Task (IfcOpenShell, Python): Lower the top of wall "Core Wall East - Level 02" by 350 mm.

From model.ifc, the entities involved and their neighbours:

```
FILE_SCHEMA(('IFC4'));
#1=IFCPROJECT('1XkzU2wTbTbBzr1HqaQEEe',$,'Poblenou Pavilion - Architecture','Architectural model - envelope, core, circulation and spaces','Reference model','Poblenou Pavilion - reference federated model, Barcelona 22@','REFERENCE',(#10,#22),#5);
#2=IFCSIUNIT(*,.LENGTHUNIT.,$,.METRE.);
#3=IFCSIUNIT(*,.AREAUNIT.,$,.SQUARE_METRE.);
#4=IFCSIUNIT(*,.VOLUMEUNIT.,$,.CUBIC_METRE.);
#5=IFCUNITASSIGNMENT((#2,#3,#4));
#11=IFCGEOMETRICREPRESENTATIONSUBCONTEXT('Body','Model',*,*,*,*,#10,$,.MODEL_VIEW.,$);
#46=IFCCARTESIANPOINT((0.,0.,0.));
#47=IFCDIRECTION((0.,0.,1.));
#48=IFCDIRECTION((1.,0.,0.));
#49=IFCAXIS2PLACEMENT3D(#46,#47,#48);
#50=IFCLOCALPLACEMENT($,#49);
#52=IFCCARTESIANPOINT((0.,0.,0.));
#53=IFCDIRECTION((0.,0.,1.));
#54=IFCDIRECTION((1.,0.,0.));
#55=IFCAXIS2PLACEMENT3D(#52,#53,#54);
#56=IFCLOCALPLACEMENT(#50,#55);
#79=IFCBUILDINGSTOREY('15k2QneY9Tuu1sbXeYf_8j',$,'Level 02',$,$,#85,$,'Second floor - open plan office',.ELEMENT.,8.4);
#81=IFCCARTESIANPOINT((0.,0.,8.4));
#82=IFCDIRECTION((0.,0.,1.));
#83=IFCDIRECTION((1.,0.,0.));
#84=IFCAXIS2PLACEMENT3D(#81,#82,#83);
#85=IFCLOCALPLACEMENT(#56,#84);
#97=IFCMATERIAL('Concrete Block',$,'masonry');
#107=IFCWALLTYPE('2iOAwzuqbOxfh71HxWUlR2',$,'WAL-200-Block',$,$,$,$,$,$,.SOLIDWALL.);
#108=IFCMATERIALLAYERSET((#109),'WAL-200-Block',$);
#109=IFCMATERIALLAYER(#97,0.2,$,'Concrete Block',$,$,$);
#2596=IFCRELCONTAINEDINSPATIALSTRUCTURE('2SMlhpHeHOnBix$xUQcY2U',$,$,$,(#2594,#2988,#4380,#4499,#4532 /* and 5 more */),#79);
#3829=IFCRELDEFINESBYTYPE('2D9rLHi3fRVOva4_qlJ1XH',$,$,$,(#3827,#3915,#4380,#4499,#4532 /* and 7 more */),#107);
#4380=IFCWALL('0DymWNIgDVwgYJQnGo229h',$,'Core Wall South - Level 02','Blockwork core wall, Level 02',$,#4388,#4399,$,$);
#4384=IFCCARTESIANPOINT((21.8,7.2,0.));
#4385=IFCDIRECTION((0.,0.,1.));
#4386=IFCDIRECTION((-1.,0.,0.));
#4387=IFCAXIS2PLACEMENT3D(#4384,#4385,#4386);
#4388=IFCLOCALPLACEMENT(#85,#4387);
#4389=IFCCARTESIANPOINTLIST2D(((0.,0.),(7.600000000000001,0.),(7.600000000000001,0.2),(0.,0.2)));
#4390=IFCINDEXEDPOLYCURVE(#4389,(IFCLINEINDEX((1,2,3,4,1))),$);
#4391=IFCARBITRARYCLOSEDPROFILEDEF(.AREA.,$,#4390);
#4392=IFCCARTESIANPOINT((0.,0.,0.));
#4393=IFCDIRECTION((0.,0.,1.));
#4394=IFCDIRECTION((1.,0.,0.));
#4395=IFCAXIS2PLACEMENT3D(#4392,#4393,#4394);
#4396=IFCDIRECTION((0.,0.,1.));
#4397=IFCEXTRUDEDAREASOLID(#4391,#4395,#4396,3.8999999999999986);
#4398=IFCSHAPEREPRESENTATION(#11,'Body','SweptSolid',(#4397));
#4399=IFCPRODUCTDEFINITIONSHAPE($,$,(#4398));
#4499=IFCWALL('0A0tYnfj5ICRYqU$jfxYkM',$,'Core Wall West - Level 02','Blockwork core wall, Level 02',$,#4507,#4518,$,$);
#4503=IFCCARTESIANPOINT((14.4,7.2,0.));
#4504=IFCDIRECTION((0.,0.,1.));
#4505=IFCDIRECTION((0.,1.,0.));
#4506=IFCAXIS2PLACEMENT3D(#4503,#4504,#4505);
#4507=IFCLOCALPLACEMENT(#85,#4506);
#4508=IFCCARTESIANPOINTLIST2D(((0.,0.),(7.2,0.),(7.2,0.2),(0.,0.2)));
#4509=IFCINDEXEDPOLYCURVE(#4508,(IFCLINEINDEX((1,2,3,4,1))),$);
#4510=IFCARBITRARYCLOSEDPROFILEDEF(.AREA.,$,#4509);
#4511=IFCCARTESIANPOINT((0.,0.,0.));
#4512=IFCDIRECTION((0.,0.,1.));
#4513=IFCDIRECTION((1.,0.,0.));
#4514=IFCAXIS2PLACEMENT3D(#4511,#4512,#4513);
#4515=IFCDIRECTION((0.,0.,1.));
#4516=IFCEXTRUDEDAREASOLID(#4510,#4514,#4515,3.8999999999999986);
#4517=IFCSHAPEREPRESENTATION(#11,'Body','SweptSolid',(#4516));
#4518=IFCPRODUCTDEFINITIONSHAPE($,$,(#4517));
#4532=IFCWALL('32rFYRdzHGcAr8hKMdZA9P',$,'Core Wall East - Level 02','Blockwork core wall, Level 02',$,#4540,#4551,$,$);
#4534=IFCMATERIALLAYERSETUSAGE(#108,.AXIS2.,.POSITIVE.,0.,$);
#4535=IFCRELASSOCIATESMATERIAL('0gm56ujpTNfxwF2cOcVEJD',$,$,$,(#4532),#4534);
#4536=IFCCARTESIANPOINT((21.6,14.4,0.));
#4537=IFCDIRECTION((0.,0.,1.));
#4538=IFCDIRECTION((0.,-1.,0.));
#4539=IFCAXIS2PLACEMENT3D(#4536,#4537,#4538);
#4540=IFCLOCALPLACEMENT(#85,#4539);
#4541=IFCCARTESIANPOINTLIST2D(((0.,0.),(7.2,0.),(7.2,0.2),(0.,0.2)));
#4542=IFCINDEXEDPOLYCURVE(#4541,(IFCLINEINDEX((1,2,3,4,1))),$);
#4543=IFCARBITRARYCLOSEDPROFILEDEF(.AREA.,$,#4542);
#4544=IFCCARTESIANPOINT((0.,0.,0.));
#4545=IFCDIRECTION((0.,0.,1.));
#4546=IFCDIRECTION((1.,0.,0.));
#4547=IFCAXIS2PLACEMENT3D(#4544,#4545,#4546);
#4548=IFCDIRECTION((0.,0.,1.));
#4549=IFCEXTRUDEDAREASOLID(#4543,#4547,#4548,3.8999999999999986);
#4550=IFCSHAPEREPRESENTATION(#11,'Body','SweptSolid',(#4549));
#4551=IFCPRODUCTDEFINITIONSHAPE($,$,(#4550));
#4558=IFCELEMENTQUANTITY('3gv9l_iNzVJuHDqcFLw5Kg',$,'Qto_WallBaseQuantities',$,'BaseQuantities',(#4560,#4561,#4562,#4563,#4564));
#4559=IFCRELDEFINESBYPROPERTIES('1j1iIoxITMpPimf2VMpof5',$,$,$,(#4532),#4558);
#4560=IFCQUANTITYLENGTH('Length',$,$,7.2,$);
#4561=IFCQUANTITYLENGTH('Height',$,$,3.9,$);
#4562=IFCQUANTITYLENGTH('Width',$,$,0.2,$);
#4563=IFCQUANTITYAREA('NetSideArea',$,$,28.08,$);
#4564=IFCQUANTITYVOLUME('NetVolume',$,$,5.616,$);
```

```python
import ifcopenshell
import ifcopenshell.api.pset
import ifcopenshell.geom
import ifcopenshell.util.element
import ifcopenshell.util.representation
import ifcopenshell.util.shape
import ifcopenshell.util.unit

model = ifcopenshell.open("model.ifc")
unit_scale = ifcopenshell.util.unit.calculate_unit_scale(model)
area_scale = ifcopenshell.util.unit.calculate_unit_scale(model, "AREAUNIT")
volume_scale = ifcopenshell.util.unit.calculate_unit_scale(model, "VOLUMEUNIT")
settings = ifcopenshell.geom.settings()


def volume(element):
    """Net volume in cubic metres, openings subtracted."""
    shape = ifcopenshell.geom.create_shape(settings, element)
    return ifcopenshell.util.shape.get_volume(shape.geometry)


wall = model.by_guid("32rFYRdzHGcAr8hKMdZA9P")
before = volume(wall)

body = ifcopenshell.util.representation.get_representation(wall, "Model", "Body")
solid = body.Items[0]
old_height = solid.Depth
solid.Depth -= 0.35 / unit_scale
after = volume(wall)
thickness = 0.2  # wall thickness in metres

# Update the stored height, areas and volumes.
qto = model.by_id(ifcopenshell.util.element.get_pset(wall, "Qto_WallBaseQuantities", should_inherit=False)["id"])
ifcopenshell.api.pset.edit_qto(model, qto=qto, properties={
    "Height": solid.Depth,
    "NetSideArea": after / thickness / area_scale,
    "NetVolume": after / volume_scale,
})

print(f"height {old_height:g} -> {solid.Depth:g}, volume {before:.3f} -> {after:.3f} m3")

model.write("model-out.ifc")
```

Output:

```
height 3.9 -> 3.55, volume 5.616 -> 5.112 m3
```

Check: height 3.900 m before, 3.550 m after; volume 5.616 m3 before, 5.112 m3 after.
